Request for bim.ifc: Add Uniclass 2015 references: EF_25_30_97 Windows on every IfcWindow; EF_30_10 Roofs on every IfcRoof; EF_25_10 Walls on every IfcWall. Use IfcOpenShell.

First a look at what the model holds.

```python
import ifcopenshell

model = ifcopenshell.open("bim.ifc")
print(model.schema)
print("classifications:", [c.Name for c in model.by_type("IfcClassification")])
for ifc_class in ("IfcDoor", "IfcRoof", "IfcStair", "IfcWall", "IfcWindow"):
    print(ifc_class, len(model.by_type(ifc_class)))
```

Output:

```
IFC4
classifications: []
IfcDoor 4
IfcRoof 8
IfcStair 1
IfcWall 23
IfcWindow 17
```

```python
import ifcopenshell
import ifcopenshell.api.classification

model = ifcopenshell.open("bim.ifc")

system = ifcopenshell.api.classification.add_classification(model, classification="Uniclass 2015")

codes = {
    "IfcWindow": ("EF_25_30_97", "Windows"),
    "IfcRoof": ("EF_30_10", "Roofs"),
    "IfcWall": ("EF_25_10", "Walls"),
}
for ifc_class, (code, name) in codes.items():
    products = model.by_type(ifc_class)
    ifcopenshell.api.classification.add_reference(
        model, products=products, classification=system, identification=code, name=name
    )
    print(code, len(products))

model.write("bim-out.ifc")
```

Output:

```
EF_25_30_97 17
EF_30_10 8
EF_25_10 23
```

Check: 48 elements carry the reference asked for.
